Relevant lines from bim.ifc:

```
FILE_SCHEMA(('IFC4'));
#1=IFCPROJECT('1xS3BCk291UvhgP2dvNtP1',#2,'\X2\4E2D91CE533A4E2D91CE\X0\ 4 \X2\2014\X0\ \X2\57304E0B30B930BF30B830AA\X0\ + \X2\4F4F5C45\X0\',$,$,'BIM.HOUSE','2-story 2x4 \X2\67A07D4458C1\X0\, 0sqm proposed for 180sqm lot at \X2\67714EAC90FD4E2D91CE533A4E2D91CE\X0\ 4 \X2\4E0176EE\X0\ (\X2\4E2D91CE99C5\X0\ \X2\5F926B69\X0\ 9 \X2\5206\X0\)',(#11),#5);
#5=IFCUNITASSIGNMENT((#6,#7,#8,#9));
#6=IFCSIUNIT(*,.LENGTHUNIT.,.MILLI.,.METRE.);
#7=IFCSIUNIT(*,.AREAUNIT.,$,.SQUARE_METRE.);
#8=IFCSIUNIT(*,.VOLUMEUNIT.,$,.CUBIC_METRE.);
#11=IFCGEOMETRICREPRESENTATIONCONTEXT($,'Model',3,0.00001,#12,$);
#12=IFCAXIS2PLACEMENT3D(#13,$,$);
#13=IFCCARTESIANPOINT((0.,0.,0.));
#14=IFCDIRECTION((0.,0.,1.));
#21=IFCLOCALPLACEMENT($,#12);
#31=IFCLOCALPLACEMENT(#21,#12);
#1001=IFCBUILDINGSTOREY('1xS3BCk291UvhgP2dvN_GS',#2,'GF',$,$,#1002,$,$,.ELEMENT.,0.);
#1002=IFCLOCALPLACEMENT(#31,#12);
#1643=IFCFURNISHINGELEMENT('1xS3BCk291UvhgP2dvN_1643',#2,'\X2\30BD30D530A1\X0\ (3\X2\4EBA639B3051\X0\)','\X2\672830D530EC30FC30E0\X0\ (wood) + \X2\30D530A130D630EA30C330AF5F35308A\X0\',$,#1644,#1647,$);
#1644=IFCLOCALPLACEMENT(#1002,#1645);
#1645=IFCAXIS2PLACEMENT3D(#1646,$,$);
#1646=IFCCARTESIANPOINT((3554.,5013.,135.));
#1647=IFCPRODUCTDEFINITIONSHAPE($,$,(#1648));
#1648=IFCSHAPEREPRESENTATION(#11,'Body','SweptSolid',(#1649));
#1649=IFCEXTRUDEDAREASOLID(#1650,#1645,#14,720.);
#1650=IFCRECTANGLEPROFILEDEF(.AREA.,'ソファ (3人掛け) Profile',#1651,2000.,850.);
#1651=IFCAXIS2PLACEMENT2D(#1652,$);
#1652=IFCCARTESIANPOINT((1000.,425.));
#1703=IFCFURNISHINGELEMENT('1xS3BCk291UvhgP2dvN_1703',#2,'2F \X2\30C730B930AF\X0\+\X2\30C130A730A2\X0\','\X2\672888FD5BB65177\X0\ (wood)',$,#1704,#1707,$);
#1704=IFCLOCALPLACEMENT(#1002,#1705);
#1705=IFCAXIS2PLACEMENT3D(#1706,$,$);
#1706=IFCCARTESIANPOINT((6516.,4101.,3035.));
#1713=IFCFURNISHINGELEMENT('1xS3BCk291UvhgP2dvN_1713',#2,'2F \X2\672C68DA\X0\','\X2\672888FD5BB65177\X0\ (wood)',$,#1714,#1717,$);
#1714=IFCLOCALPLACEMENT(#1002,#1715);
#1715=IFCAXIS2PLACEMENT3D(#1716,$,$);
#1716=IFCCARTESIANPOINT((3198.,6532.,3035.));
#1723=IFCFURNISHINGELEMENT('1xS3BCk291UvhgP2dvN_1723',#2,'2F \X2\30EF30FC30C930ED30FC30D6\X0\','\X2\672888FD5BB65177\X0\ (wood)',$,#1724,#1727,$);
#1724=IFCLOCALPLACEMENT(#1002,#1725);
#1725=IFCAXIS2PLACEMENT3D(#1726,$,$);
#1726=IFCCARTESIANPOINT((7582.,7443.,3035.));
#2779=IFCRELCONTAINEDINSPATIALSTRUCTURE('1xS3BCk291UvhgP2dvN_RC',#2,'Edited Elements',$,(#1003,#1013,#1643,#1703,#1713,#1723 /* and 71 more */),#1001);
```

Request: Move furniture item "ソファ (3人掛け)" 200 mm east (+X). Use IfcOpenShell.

```python
import ifcopenshell
import ifcopenshell.api.geometry
import ifcopenshell.util.placement
import ifcopenshell.util.unit

model = ifcopenshell.open("bim.ifc")
unit_scale = ifcopenshell.util.unit.calculate_unit_scale(model)

item = model.by_guid("1xS3BCk291UvhgP2dvN_1643")
matrix = ifcopenshell.util.placement.get_local_placement(item.ObjectPlacement)
matrix[0, 3] += 0.2 / unit_scale
ifcopenshell.api.geometry.edit_object_placement(model, product=item, matrix=matrix, is_si=False)

print(ifcopenshell.util.placement.get_local_placement(item.ObjectPlacement).round(3) + 0.0)

model.write("bim_v2.ifc")
```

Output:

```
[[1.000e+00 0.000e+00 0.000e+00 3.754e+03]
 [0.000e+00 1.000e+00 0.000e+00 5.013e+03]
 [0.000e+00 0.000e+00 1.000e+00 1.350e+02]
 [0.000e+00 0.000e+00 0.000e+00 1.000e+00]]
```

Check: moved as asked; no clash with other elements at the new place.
